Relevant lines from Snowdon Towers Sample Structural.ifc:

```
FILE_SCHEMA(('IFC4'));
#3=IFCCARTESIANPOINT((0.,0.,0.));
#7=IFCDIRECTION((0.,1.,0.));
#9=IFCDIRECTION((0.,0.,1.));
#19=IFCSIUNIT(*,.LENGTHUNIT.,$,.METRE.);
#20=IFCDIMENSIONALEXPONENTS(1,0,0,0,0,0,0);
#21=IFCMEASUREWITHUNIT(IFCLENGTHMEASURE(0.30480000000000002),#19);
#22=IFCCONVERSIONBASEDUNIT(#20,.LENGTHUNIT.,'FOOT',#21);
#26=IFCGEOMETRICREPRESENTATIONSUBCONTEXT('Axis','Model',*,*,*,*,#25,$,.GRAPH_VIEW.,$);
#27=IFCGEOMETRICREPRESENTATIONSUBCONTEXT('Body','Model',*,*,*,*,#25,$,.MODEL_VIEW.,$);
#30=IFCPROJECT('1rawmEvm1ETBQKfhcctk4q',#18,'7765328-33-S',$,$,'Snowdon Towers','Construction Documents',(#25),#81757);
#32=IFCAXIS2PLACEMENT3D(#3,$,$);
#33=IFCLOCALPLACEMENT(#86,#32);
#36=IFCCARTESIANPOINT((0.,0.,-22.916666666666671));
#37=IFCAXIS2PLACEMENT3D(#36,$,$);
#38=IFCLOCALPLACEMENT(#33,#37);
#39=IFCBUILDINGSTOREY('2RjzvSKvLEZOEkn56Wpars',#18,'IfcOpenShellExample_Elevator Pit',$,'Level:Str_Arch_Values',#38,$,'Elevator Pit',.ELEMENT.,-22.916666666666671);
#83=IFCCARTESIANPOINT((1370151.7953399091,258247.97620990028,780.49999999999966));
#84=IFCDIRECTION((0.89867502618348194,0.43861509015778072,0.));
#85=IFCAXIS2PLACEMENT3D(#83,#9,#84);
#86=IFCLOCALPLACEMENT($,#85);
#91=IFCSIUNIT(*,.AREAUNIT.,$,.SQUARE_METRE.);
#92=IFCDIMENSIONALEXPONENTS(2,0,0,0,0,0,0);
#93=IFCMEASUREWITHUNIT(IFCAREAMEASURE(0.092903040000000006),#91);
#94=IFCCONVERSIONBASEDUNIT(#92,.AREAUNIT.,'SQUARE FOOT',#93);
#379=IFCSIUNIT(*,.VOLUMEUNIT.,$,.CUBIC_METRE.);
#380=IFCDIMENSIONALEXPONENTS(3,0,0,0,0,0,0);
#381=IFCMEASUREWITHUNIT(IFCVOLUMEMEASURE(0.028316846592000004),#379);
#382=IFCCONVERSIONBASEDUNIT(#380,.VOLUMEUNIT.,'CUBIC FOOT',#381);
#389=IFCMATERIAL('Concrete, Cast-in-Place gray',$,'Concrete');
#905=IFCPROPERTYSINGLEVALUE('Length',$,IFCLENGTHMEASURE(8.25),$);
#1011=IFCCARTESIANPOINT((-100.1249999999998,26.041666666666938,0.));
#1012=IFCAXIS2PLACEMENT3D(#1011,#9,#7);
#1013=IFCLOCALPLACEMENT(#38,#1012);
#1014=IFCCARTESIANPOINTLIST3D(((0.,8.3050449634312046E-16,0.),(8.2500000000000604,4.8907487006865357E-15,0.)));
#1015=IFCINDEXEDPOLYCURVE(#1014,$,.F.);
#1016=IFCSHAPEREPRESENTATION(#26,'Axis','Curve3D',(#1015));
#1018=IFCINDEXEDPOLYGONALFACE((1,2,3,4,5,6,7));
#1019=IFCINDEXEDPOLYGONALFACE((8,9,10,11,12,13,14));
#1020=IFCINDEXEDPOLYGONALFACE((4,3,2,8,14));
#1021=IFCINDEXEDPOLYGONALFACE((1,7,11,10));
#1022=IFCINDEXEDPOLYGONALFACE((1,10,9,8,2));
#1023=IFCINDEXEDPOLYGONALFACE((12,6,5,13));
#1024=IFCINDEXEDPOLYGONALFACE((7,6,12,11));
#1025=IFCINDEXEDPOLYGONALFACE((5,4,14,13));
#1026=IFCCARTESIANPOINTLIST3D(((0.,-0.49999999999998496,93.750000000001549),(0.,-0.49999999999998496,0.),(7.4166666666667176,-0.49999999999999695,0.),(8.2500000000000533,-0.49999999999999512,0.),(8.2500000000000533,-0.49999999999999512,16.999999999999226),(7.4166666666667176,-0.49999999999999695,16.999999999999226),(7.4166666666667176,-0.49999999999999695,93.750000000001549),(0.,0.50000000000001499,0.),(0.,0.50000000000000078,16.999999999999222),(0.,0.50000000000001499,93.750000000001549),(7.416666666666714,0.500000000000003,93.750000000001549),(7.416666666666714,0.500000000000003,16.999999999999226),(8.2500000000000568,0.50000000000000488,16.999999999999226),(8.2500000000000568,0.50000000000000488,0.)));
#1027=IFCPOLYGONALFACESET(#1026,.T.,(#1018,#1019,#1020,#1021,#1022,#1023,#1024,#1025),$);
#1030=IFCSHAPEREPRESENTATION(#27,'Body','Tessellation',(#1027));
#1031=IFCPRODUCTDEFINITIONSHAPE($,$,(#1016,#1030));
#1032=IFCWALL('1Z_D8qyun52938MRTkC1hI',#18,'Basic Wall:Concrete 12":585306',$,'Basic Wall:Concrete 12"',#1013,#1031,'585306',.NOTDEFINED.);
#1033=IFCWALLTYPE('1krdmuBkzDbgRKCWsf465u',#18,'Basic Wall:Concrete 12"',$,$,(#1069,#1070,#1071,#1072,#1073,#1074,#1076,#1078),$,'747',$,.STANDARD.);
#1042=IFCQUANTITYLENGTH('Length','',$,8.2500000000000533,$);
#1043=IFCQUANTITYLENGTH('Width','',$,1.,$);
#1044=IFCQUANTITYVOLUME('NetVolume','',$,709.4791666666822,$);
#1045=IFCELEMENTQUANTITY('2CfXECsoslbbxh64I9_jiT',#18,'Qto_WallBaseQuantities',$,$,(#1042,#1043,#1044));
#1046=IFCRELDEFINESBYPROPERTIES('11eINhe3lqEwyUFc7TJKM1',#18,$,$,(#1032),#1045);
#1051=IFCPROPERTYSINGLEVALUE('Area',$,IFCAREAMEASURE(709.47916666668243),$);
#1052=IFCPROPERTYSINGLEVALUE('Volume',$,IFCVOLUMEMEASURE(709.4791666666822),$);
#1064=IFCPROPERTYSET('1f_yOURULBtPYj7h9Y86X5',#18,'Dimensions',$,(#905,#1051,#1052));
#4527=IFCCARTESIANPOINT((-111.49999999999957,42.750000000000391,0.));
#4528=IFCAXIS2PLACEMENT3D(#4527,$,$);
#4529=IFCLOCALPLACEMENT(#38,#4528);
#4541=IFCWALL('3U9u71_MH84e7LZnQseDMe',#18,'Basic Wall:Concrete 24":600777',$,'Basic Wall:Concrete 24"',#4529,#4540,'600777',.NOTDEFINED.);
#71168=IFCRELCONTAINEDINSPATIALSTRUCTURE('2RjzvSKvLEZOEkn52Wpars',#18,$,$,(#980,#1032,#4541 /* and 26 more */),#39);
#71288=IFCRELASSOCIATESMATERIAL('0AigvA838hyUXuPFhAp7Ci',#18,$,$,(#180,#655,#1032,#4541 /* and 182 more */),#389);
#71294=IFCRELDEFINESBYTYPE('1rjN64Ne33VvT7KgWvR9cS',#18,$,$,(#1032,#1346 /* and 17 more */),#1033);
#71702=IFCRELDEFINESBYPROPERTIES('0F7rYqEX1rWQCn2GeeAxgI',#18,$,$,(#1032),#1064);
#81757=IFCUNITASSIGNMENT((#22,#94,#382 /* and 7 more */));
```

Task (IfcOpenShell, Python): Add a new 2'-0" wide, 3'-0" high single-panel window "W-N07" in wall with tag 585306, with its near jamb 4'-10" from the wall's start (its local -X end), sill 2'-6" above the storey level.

```python
import numpy as np
import ifcopenshell
import ifcopenshell.api.feature
import ifcopenshell.api.geometry
import ifcopenshell.api.pset
import ifcopenshell.api.root
import ifcopenshell.api.spatial
import ifcopenshell.geom
import ifcopenshell.util.element
import ifcopenshell.util.placement
import ifcopenshell.util.representation
import ifcopenshell.util.shape
import ifcopenshell.util.unit

model = ifcopenshell.open("Snowdon Towers Sample Structural.ifc")
unit_scale = ifcopenshell.util.unit.calculate_unit_scale(model)
area_scale = ifcopenshell.util.unit.calculate_unit_scale(model, "AREAUNIT")
volume_scale = ifcopenshell.util.unit.calculate_unit_scale(model, "VOLUMEUNIT")
settings = ifcopenshell.geom.settings()


def volume(element):
    """Net volume in cubic metres, openings subtracted."""
    shape = ifcopenshell.geom.create_shape(settings, element)
    return ifcopenshell.util.shape.get_volume(shape.geometry)


wall = model.by_guid("1Z_D8qyun52938MRTkC1hI")
storey = ifcopenshell.util.element.get_container(wall, ifc_class="IfcBuildingStorey")
context = ifcopenshell.util.representation.get_context(model, "Model", "Body", "MODEL_VIEW")
before = volume(wall)

width, height, from_end, sill = 0.6096, 0.9144, 1.4732, 0.762  # metres

# The wall runs along its own X axis, and the end named is its -X end.
wall_shape = ifcopenshell.geom.create_shape(settings, wall)
x, y, z = ifcopenshell.util.shape.get_vertices(wall_shape.geometry).T
start = x.min() + from_end
face, thickness = float(y.min()), float(y.max() - y.min())
wall_matrix = ifcopenshell.util.placement.get_local_placement(wall.ObjectPlacement)
level = ifcopenshell.util.placement.get_local_placement(storey.ObjectPlacement)[2, 3]


def in_wall(x, y):
    """Placement at x, y metres in the wall's axes, at sill height."""
    matrix = wall_matrix.copy()
    matrix[:, 3] = wall_matrix @ np.array([x / unit_scale, y / unit_scale, 0.0, 1.0])
    matrix[2, 3] = level + sill / unit_scale
    return matrix


# Opening: a box that overshoots both wall faces by 50 mm.
opening = ifcopenshell.api.root.create_entity(model, ifc_class="IfcOpeningElement", predefined_type="OPENING")
box = ifcopenshell.api.geometry.add_wall_representation(
    model, context=context, length=width, height=height, thickness=thickness + 0.1
)
ifcopenshell.api.geometry.assign_representation(model, product=opening, representation=box)
ifcopenshell.api.geometry.edit_object_placement(model, product=opening, matrix=in_wall(start, face - 0.05), is_si=False)
ifcopenshell.api.feature.add_feature(model, feature=opening, element=wall)

window = ifcopenshell.api.root.create_entity(model, ifc_class="IfcWindow", name="W-N07", predefined_type="WINDOW")
window.OverallWidth, window.OverallHeight = width / unit_scale, height / unit_scale
window.PartitioningType = "SINGLE_PANEL"
body = ifcopenshell.api.geometry.add_window_representation(
    model,
    context=context,
    overall_width=window.OverallWidth,
    overall_height=window.OverallHeight,
    partition_type="SINGLE_PANEL",
)
ifcopenshell.api.geometry.assign_representation(model, product=window, representation=body)
ifcopenshell.api.spatial.assign_container(model, products=[window], relating_structure=storey)
ifcopenshell.api.feature.add_filling(model, opening=opening, element=window)

# Centre the window in the wall's thickness.
ifcopenshell.api.geometry.edit_object_placement(model, product=window, matrix=in_wall(start, face), is_si=False)
window_shape = ifcopenshell.geom.create_shape(settings, window)
depth = ifcopenshell.util.shape.get_vertices(window_shape.geometry)[:, 1]
offset = face + thickness / 2 - (depth.min() + depth.max()) / 2
ifcopenshell.api.geometry.edit_object_placement(model, product=window, matrix=in_wall(start, offset), is_si=False)

after = volume(wall)

# Update the wall's stored quantities.
qto = model.by_id(ifcopenshell.util.element.get_pset(wall, "Qto_WallBaseQuantities", should_inherit=False)["id"])
ifcopenshell.api.pset.edit_qto(model, qto=qto, properties={"NetVolume": after / volume_scale})
pset = model.by_id(ifcopenshell.util.element.get_pset(wall, "Dimensions", should_inherit=False)["id"])
ifcopenshell.api.pset.edit_pset(model, pset=pset, properties={
    "Area": model.create_entity("IfcAreaMeasure", after / thickness / area_scale),
    "Volume": model.create_entity("IfcVolumeMeasure", after / volume_scale),
})

print(f"wall volume {before:.3f} -> {after:.3f} m3")

model.write("Snowdon Towers Sample Structural_rev.ifc")
```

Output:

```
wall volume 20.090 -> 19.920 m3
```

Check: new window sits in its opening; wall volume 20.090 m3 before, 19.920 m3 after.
